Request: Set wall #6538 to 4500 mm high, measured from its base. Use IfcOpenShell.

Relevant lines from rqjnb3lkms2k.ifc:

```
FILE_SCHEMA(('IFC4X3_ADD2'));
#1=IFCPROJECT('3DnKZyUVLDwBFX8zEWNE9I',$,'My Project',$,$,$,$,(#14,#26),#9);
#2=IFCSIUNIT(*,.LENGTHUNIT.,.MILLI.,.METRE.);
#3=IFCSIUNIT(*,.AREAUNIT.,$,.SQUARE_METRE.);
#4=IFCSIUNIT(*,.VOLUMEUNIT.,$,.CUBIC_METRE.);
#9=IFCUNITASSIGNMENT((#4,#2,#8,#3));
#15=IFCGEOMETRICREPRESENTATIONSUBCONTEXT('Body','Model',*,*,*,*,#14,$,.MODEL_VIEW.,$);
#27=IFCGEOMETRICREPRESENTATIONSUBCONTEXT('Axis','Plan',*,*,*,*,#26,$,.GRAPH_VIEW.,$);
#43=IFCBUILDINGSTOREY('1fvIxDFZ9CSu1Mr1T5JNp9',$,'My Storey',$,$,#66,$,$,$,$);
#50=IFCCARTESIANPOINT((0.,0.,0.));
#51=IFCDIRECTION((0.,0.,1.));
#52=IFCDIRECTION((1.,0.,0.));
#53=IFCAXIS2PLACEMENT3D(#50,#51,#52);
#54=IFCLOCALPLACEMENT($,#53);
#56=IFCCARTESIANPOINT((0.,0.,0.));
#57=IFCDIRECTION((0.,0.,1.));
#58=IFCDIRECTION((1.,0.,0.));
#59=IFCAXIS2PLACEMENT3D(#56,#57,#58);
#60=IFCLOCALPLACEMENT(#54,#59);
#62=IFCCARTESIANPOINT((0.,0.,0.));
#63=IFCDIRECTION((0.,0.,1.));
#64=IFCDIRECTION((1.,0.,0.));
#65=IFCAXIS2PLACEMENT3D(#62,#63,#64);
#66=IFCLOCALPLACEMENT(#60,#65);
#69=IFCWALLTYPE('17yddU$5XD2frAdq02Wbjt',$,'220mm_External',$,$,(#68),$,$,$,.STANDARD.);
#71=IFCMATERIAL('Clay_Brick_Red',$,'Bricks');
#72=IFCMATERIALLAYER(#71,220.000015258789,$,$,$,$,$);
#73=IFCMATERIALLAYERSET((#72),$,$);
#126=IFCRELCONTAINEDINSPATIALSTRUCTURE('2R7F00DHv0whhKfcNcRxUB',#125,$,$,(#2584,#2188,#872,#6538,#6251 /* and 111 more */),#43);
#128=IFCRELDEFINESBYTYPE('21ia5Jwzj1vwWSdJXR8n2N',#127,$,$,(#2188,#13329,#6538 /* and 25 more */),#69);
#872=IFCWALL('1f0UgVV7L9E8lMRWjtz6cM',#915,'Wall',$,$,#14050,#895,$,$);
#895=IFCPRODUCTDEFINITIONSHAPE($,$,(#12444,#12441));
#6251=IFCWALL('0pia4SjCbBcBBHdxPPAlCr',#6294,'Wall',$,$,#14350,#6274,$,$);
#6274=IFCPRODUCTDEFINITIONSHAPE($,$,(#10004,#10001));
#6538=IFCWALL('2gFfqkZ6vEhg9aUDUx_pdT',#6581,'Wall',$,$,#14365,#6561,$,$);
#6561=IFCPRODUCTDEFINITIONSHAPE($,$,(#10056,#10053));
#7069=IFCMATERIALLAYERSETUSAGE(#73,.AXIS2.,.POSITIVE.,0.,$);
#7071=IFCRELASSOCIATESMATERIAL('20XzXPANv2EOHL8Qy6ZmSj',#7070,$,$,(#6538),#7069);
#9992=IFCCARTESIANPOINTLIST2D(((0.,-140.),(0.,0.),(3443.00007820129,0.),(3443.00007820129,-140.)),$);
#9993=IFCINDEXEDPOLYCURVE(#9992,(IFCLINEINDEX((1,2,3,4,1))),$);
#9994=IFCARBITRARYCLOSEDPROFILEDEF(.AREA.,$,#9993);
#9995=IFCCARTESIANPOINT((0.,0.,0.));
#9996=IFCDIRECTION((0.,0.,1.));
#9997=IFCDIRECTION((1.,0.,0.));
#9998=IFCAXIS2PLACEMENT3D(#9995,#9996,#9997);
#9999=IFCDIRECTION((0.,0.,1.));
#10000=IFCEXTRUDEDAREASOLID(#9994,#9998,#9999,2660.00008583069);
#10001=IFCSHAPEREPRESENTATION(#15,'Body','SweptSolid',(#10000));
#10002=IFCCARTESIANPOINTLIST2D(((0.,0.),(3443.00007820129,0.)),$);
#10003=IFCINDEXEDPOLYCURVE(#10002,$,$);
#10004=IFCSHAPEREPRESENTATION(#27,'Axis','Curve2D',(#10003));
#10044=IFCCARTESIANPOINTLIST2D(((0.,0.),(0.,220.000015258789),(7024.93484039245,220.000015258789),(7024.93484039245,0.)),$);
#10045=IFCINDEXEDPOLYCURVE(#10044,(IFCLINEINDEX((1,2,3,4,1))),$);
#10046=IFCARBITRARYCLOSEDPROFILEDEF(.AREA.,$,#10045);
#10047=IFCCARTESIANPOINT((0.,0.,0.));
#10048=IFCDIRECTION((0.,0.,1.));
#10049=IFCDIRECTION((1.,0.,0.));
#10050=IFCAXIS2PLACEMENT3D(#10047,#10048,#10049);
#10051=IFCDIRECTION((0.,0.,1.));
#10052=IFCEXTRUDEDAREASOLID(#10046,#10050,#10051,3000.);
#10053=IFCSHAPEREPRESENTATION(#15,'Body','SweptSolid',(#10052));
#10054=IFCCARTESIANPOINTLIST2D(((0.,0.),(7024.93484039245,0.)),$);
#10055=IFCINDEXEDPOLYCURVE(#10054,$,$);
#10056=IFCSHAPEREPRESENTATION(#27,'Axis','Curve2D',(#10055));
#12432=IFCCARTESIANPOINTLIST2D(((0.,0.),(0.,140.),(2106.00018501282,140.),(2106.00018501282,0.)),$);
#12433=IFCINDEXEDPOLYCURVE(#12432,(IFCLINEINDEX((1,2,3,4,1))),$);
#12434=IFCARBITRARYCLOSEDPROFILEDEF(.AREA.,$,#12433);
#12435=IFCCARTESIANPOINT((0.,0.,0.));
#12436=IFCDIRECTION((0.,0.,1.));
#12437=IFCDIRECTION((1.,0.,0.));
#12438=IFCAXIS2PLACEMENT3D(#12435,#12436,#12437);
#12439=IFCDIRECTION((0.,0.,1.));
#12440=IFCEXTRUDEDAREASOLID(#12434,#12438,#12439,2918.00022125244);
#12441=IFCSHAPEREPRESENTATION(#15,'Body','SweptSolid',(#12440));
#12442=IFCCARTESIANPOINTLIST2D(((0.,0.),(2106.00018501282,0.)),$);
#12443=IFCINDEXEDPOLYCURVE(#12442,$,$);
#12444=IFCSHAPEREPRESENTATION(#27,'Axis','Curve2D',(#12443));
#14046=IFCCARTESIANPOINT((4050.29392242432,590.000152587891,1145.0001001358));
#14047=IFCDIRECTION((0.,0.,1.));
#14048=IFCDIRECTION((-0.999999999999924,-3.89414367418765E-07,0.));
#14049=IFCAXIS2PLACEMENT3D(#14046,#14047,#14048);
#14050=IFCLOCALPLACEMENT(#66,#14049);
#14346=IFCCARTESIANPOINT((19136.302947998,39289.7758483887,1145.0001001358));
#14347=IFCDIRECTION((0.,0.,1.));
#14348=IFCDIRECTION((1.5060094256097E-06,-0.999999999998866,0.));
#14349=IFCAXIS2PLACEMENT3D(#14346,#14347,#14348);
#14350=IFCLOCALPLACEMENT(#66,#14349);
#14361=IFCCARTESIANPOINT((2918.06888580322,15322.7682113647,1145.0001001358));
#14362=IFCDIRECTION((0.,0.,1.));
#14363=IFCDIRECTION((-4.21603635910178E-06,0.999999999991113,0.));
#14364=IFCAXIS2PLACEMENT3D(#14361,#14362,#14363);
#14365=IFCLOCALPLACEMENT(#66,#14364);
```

```python
import ifcopenshell
import ifcopenshell.geom
import ifcopenshell.util.representation
import ifcopenshell.util.shape
import ifcopenshell.util.unit

model = ifcopenshell.open("rqjnb3lkms2k.ifc")
unit_scale = ifcopenshell.util.unit.calculate_unit_scale(model)
settings = ifcopenshell.geom.settings()


def volume(element):
    """Net volume in cubic metres, openings subtracted."""
    shape = ifcopenshell.geom.create_shape(settings, element)
    return ifcopenshell.util.shape.get_volume(shape.geometry)


wall = model.by_id(6538)
before = volume(wall)

body = ifcopenshell.util.representation.get_representation(wall, "Model", "Body")
solid = body.Items[0]
old_height = solid.Depth
solid.Depth = 4.5 / unit_scale
after = volume(wall)

print(f"height {old_height:g} -> {solid.Depth:g}, volume {before:.3f} -> {after:.3f} m3")

model.write("rqjnb3lkms2k_v2.ifc")
```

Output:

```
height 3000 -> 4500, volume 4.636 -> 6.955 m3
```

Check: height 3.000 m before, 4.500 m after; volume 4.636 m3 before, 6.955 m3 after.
